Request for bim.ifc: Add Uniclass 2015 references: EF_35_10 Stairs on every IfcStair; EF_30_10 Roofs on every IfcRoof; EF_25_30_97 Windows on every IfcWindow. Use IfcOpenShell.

First a look at what the model holds.

```python
import ifcopenshell

model = ifcopenshell.open("bim.ifc")
print(model.schema)
print("classifications:", [c.Name for c in model.by_type("IfcClassification")])
for ifc_class in ("IfcDoor", "IfcRoof", "IfcStair", "IfcWall", "IfcWindow"):
    print(ifc_class, len(model.by_type(ifc_class)))
```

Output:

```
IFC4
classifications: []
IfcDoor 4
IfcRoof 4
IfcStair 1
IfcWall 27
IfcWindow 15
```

```python
import ifcopenshell
import ifcopenshell.api.classification

model = ifcopenshell.open("bim.ifc")

system = ifcopenshell.api.classification.add_classification(model, classification="Uniclass 2015")

codes = {
    "IfcStair": ("EF_35_10", "Stairs"),
    "IfcRoof": ("EF_30_10", "Roofs"),
    "IfcWindow": ("EF_25_30_97", "Windows"),
}
for ifc_class, (code, name) in codes.items():
    products = model.by_type(ifc_class)
    ifcopenshell.api.classification.add_reference(
        model, products=products, classification=system, identification=code, name=name
    )
    print(code, len(products))

model.write("bim-out.ifc")
```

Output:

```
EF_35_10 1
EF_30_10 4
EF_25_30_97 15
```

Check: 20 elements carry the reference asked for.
